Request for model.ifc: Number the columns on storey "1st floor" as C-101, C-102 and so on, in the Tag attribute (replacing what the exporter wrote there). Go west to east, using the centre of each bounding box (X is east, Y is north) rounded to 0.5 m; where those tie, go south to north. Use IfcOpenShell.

First a look at what the model holds.

```python
import ifcopenshell
import ifcopenshell.util.element
import ifcopenshell.util.placement

model = ifcopenshell.open("model.ifc")
print(model.schema)
storey = next(s for s in model.by_type("IfcBuildingStorey") if s.Name == "1st floor")
columns = [e for e in ifcopenshell.util.element.get_decomposition(storey) if e.is_a("IfcColumn")]
for e in sorted(columns, key=lambda e: e.id()):
    origin = ifcopenshell.util.placement.get_local_placement(e.ObjectPlacement)[:3, 3]
    print(e.id(), e.Tag, e.Name, origin.round(2) + 0.0, sep=" | ")
```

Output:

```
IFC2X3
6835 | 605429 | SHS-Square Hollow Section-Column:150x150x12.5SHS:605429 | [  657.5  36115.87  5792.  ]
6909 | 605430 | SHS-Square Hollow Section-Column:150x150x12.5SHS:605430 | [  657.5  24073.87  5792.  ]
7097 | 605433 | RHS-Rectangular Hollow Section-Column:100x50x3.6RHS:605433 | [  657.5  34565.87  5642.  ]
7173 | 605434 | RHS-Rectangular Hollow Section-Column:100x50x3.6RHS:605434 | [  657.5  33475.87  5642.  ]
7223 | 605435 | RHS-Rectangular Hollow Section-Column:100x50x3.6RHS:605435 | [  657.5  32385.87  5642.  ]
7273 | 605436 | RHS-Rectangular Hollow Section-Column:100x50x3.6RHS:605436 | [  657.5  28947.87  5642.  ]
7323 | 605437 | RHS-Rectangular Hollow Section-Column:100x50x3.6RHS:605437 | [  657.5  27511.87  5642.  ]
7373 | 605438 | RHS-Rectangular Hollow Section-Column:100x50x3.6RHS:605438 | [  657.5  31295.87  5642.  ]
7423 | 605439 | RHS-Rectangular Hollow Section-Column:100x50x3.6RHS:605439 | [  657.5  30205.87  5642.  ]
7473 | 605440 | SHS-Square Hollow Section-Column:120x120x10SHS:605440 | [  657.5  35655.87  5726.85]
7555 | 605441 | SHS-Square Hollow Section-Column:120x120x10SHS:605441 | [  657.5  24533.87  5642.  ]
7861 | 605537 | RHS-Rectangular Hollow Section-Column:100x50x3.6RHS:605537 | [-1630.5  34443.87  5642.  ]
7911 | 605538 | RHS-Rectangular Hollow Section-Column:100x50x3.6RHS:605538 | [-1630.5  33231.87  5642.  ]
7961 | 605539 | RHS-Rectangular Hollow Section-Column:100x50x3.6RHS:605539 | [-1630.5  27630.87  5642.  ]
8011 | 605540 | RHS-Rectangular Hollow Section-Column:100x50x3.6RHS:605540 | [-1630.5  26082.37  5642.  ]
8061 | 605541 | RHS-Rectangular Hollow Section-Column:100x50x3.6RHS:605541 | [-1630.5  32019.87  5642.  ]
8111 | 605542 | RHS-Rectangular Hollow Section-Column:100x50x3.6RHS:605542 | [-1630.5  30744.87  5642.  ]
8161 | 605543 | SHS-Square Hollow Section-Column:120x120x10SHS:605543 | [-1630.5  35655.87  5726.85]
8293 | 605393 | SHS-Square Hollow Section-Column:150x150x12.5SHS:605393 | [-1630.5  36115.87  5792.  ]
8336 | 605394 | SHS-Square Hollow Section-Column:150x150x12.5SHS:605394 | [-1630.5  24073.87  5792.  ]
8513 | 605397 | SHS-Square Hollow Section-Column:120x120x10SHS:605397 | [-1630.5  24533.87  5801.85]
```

```python
import ifcopenshell
import ifcopenshell.geom
import ifcopenshell.util.element
import ifcopenshell.util.shape

model = ifcopenshell.open("model.ifc")
settings = ifcopenshell.geom.settings()
settings.set("use-world-coords", True)


def centre(element):
    shape = ifcopenshell.geom.create_shape(settings, element)
    return ifcopenshell.util.shape.get_bbox_centroid(shape.geometry)


storey = next(s for s in model.by_type("IfcBuildingStorey") if s.Name == "1st floor")
columns = [e for e in ifcopenshell.util.element.get_decomposition(storey) if e.is_a("IfcColumn")]

# Insertion points can sit at a corner or the storey origin, so sort by the geometry (in metres).
centres = {e: centre(e) for e in columns}
columns.sort(key=lambda e: (round(centres[e][0] / 0.5), centres[e][1]))

for i, e in enumerate(columns, start=1):
    number = f"C-1{i:02d}"
    e.Tag = number
    print(e.id(), number)

model.write("model_edited.ifc")
```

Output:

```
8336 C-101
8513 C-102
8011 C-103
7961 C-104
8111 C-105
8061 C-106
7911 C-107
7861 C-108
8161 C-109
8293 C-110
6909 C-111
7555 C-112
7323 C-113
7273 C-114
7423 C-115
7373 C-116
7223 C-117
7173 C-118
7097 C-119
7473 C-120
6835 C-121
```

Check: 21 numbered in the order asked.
